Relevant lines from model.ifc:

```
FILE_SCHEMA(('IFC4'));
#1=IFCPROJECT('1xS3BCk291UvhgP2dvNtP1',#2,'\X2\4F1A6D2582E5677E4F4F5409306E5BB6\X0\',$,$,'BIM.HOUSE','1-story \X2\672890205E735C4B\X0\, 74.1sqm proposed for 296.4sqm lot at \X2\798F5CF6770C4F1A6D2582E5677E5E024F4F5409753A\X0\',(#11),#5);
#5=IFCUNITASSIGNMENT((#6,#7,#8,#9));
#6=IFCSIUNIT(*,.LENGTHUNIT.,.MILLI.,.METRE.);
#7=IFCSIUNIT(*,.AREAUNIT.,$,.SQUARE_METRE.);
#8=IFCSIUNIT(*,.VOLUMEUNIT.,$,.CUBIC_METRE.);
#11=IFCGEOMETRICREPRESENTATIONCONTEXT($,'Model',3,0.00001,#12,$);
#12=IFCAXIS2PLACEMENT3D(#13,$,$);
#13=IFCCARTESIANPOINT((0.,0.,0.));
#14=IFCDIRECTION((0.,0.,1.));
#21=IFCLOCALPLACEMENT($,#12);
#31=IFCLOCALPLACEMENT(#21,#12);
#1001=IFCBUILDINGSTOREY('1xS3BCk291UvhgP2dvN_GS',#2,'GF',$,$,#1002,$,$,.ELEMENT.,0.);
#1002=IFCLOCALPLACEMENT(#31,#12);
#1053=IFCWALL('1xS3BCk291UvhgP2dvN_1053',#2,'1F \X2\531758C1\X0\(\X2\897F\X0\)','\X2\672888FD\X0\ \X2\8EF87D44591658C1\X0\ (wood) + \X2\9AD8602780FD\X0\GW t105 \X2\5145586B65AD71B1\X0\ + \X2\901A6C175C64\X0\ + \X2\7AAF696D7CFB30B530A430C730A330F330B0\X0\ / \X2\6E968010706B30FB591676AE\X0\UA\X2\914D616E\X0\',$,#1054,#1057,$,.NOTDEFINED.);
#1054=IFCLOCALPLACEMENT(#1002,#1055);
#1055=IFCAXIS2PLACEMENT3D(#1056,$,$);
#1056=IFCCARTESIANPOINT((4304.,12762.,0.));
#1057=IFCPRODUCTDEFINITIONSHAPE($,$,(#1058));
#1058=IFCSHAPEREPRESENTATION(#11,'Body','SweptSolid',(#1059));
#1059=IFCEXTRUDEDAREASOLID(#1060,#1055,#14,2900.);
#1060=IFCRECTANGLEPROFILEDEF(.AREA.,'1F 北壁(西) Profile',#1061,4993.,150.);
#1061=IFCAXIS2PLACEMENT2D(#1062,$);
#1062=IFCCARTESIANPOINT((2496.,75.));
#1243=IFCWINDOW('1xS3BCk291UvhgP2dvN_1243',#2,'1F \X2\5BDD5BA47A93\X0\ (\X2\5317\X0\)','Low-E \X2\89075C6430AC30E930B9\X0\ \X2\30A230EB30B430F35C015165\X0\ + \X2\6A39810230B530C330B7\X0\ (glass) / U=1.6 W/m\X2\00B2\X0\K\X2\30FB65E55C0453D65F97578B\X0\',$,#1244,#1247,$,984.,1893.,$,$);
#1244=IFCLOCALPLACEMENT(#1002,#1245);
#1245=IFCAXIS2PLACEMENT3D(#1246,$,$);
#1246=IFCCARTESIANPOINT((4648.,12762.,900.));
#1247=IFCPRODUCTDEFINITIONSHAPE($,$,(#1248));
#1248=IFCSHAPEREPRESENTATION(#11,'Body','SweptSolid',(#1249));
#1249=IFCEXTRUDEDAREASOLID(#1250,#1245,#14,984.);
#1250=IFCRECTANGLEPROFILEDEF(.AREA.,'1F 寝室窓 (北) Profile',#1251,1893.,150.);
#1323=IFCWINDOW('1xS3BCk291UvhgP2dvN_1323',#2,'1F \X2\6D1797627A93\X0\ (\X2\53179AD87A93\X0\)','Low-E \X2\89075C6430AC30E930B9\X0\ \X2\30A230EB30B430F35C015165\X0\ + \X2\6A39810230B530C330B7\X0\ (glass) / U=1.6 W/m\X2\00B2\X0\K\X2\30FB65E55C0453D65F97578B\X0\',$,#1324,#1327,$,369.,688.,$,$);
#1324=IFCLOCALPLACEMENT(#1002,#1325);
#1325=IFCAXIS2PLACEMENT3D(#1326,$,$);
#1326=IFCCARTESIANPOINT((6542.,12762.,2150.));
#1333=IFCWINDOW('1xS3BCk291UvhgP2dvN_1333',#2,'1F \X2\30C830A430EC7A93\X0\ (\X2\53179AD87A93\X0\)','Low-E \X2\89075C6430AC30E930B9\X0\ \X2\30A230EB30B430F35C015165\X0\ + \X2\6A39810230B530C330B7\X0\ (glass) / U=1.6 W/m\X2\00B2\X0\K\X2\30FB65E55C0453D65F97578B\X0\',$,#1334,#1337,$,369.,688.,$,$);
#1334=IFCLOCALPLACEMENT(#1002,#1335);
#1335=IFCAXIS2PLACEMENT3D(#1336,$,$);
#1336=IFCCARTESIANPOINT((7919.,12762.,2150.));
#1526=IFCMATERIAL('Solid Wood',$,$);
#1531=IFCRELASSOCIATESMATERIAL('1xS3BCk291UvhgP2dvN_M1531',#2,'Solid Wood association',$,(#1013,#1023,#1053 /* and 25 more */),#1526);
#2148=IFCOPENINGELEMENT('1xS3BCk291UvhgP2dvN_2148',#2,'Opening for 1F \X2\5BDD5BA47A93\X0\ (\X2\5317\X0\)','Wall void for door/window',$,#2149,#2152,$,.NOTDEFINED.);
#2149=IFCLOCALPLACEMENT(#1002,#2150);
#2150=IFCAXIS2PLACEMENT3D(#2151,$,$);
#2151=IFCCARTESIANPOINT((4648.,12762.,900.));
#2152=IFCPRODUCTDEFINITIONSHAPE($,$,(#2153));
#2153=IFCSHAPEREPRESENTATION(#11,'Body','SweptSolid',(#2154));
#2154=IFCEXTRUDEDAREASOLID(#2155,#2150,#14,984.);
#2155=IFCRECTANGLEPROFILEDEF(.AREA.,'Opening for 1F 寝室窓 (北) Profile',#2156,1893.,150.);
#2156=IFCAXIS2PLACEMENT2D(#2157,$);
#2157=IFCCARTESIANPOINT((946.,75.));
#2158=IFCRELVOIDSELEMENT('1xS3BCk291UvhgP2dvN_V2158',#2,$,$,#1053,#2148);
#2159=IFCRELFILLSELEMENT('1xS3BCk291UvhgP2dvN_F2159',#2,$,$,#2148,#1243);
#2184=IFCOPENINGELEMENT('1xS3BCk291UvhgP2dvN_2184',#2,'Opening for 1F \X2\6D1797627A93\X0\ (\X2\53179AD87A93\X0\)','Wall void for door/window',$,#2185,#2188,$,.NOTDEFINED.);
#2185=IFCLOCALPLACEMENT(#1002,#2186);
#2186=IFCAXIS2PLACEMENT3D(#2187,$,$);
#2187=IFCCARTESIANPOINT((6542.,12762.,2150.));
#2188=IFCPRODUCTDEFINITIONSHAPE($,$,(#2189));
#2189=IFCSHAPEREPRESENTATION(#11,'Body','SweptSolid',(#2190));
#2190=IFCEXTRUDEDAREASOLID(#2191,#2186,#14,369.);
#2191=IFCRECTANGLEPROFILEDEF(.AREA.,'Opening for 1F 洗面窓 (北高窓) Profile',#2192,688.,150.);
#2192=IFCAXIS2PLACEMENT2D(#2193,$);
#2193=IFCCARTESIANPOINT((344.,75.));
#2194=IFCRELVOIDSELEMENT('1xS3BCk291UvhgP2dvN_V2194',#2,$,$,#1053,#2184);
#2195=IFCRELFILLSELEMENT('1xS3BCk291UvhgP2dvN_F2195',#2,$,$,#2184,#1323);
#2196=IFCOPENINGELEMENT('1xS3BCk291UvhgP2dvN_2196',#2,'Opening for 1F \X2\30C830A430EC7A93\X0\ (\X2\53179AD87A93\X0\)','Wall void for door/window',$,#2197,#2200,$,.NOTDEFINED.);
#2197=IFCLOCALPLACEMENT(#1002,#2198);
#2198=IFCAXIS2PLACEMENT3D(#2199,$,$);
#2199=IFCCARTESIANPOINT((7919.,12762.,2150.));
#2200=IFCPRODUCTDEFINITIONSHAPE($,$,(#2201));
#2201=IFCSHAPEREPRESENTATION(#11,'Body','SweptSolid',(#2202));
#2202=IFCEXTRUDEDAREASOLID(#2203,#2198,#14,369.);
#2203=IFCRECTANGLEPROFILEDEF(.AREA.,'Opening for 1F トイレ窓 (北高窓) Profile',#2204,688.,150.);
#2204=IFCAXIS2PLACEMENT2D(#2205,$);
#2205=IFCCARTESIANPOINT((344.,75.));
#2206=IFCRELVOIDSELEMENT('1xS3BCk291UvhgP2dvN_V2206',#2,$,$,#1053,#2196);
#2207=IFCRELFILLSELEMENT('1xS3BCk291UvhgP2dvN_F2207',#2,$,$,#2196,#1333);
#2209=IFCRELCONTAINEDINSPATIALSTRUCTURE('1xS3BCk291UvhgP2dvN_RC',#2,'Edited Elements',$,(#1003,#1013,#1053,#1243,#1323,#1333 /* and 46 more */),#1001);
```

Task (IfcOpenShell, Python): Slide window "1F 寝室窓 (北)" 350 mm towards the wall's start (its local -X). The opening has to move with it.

```python
import ifcopenshell
import ifcopenshell.api.geometry
import ifcopenshell.util.placement
import ifcopenshell.util.unit

model = ifcopenshell.open("model.ifc")
unit_scale = ifcopenshell.util.unit.calculate_unit_scale(model)

window = model.by_guid("1xS3BCk291UvhgP2dvN_1243")
opening = window.FillsVoids[0].RelatingOpeningElement
wall = opening.VoidsElements[0].RelatingBuildingElement

wall_matrix = ifcopenshell.util.placement.get_local_placement(wall.ObjectPlacement)
shift = wall_matrix[:3, 0] * -0.35 / unit_scale
before = ifcopenshell.util.placement.get_local_placement(window.ObjectPlacement)[:3, 3].copy()

# The window is not placed relative to its opening, so move both.
for product in (opening, window):
    matrix = ifcopenshell.util.placement.get_local_placement(product.ObjectPlacement)
    matrix[:3, 3] += shift
    ifcopenshell.api.geometry.edit_object_placement(model, product=product, matrix=matrix, is_si=False)

after = ifcopenshell.util.placement.get_local_placement(window.ObjectPlacement)[:3, 3]
print("window moved by", (after - before).round(3) + 0.0)

model.write("model_rev.ifc")
```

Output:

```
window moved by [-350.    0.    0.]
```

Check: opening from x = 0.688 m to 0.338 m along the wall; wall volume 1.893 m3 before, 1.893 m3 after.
